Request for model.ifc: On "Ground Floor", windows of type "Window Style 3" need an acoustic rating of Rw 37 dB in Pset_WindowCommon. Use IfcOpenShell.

First a look at what the model holds.

```python
import ifcopenshell
import ifcopenshell.util.element

model = ifcopenshell.open("model.ifc")
print(model.schema)
storey = next(s for s in model.by_type("IfcBuildingStorey") if s.Name == "Ground Floor")
windows = [e for e in ifcopenshell.util.element.get_decomposition(storey) if e.is_a("IfcWindow")]
seen = {}
for e in windows:
    element_type = ifcopenshell.util.element.get_type(e)
    key = (element_type.Name if element_type != e and element_type else None, ifcopenshell.util.element.get_pset(e, "Pset_WindowCommon", "AcousticRating"))
    seen[key] = seen.get(key, 0) + 1
for (name, value), count in sorted(seen.items(), key=str):
    print(count, "x", name, "|", value)
```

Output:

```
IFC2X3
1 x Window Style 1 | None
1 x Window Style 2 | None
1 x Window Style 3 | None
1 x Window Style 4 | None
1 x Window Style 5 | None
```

```python
import ifcopenshell
import ifcopenshell.api.pset
import ifcopenshell.util.element

model = ifcopenshell.open("model.ifc")

storey = next(s for s in model.by_type("IfcBuildingStorey") if s.Name == "Ground Floor")
windows = [e for e in ifcopenshell.util.element.get_decomposition(storey) if e.is_a("IfcWindow")]

count = 0
for e in windows:
    element_type = ifcopenshell.util.element.get_type(e)
    if element_type in (None, e) or element_type.Name != "Window Style 3":
        continue
    # add_pset returns the element's existing set when there is one.
    pset = ifcopenshell.api.pset.add_pset(model, product=e, name="Pset_WindowCommon")
    ifcopenshell.api.pset.edit_pset(model, pset=pset, properties={"AcousticRating": "Rw 37 dB"})
    count += 1

print(count, "windows updated")

model.write("model_rev.ifc")
```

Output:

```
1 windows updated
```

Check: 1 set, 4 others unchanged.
